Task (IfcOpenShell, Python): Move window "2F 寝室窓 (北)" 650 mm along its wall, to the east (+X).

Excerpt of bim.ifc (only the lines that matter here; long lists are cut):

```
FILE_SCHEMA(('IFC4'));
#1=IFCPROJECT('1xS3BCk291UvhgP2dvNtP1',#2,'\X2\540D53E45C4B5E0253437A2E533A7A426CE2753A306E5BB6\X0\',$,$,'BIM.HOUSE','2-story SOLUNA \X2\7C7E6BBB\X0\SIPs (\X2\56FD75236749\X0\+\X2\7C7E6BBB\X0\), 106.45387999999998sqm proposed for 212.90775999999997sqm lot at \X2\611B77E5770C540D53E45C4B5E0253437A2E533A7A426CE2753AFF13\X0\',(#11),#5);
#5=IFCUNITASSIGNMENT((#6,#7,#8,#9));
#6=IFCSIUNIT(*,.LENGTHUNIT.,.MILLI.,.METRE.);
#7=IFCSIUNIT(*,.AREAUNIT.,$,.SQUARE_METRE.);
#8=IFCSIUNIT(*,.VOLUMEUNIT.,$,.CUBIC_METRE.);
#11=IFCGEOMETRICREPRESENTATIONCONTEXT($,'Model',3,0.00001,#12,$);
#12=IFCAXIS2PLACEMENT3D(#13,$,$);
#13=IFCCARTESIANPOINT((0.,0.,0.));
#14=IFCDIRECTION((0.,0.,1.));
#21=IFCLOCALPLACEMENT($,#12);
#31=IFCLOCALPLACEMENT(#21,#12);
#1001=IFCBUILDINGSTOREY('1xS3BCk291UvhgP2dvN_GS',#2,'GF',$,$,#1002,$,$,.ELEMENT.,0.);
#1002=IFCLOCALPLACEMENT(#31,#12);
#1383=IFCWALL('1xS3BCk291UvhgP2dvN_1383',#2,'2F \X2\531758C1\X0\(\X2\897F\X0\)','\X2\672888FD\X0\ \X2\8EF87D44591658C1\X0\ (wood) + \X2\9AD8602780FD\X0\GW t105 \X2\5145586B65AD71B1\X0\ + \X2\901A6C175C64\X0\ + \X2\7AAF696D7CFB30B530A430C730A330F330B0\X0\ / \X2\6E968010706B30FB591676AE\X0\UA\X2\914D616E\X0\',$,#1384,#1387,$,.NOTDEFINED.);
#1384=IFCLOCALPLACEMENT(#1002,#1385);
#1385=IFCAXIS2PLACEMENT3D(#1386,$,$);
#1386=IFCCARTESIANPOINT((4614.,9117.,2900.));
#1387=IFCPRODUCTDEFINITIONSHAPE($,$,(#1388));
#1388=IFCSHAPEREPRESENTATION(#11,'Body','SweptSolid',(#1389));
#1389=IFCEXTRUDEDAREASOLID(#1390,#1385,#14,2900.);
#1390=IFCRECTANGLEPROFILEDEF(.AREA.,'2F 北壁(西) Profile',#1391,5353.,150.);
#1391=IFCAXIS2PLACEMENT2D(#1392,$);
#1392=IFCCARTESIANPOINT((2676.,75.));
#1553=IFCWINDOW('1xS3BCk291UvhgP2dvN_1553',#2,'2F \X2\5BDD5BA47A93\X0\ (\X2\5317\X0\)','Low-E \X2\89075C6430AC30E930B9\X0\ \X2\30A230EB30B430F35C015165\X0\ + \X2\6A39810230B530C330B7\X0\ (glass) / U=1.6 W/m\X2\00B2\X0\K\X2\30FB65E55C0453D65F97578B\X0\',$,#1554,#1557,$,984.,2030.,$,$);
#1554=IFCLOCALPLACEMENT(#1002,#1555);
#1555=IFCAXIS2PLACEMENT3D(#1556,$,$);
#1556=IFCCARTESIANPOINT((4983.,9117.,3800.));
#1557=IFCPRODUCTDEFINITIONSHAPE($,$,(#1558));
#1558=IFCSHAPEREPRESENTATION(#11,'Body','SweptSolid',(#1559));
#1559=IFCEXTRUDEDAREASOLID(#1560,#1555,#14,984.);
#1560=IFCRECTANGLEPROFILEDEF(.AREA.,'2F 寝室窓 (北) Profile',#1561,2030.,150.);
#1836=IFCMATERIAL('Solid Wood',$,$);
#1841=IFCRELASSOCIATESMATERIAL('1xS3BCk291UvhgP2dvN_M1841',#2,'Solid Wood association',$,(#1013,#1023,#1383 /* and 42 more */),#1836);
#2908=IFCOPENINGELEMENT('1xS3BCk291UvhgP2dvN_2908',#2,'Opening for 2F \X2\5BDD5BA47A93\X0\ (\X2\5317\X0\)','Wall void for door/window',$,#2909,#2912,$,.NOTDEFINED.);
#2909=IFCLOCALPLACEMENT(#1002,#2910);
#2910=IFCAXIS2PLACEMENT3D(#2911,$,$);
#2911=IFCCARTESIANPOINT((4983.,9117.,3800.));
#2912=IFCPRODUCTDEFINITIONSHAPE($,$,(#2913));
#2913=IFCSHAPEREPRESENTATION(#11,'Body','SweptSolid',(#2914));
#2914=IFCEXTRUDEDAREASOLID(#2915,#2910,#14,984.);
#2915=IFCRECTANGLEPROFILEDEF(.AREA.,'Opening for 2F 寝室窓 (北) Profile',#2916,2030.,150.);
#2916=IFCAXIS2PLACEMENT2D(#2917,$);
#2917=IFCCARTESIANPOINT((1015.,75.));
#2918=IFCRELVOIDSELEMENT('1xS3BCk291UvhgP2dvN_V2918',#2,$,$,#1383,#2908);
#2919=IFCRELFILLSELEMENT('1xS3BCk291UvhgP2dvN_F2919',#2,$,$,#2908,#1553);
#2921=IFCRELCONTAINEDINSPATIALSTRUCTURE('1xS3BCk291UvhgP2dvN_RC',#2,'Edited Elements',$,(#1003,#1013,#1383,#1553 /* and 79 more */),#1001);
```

```python
import ifcopenshell
import ifcopenshell.api.geometry
import ifcopenshell.util.placement
import ifcopenshell.util.unit

model = ifcopenshell.open("bim.ifc")
unit_scale = ifcopenshell.util.unit.calculate_unit_scale(model)

window = model.by_guid("1xS3BCk291UvhgP2dvN_1553")
opening = window.FillsVoids[0].RelatingOpeningElement
wall = opening.VoidsElements[0].RelatingBuildingElement

wall_matrix = ifcopenshell.util.placement.get_local_placement(wall.ObjectPlacement)
shift = wall_matrix[:3, 0] * 0.65 / unit_scale
before = ifcopenshell.util.placement.get_local_placement(window.ObjectPlacement)[:3, 3].copy()

# The window is not placed relative to its opening, so move both.
for product in (opening, window):
    matrix = ifcopenshell.util.placement.get_local_placement(product.ObjectPlacement)
    matrix[:3, 3] += shift
    ifcopenshell.api.geometry.edit_object_placement(model, product=product, matrix=matrix, is_si=False)

after = ifcopenshell.util.placement.get_local_placement(window.ObjectPlacement)[:3, 3]
print("window moved by", (after - before).round(3) + 0.0)

model.write("bim_v2.ifc")
```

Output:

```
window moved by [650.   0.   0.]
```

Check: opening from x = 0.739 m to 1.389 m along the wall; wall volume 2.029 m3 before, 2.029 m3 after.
